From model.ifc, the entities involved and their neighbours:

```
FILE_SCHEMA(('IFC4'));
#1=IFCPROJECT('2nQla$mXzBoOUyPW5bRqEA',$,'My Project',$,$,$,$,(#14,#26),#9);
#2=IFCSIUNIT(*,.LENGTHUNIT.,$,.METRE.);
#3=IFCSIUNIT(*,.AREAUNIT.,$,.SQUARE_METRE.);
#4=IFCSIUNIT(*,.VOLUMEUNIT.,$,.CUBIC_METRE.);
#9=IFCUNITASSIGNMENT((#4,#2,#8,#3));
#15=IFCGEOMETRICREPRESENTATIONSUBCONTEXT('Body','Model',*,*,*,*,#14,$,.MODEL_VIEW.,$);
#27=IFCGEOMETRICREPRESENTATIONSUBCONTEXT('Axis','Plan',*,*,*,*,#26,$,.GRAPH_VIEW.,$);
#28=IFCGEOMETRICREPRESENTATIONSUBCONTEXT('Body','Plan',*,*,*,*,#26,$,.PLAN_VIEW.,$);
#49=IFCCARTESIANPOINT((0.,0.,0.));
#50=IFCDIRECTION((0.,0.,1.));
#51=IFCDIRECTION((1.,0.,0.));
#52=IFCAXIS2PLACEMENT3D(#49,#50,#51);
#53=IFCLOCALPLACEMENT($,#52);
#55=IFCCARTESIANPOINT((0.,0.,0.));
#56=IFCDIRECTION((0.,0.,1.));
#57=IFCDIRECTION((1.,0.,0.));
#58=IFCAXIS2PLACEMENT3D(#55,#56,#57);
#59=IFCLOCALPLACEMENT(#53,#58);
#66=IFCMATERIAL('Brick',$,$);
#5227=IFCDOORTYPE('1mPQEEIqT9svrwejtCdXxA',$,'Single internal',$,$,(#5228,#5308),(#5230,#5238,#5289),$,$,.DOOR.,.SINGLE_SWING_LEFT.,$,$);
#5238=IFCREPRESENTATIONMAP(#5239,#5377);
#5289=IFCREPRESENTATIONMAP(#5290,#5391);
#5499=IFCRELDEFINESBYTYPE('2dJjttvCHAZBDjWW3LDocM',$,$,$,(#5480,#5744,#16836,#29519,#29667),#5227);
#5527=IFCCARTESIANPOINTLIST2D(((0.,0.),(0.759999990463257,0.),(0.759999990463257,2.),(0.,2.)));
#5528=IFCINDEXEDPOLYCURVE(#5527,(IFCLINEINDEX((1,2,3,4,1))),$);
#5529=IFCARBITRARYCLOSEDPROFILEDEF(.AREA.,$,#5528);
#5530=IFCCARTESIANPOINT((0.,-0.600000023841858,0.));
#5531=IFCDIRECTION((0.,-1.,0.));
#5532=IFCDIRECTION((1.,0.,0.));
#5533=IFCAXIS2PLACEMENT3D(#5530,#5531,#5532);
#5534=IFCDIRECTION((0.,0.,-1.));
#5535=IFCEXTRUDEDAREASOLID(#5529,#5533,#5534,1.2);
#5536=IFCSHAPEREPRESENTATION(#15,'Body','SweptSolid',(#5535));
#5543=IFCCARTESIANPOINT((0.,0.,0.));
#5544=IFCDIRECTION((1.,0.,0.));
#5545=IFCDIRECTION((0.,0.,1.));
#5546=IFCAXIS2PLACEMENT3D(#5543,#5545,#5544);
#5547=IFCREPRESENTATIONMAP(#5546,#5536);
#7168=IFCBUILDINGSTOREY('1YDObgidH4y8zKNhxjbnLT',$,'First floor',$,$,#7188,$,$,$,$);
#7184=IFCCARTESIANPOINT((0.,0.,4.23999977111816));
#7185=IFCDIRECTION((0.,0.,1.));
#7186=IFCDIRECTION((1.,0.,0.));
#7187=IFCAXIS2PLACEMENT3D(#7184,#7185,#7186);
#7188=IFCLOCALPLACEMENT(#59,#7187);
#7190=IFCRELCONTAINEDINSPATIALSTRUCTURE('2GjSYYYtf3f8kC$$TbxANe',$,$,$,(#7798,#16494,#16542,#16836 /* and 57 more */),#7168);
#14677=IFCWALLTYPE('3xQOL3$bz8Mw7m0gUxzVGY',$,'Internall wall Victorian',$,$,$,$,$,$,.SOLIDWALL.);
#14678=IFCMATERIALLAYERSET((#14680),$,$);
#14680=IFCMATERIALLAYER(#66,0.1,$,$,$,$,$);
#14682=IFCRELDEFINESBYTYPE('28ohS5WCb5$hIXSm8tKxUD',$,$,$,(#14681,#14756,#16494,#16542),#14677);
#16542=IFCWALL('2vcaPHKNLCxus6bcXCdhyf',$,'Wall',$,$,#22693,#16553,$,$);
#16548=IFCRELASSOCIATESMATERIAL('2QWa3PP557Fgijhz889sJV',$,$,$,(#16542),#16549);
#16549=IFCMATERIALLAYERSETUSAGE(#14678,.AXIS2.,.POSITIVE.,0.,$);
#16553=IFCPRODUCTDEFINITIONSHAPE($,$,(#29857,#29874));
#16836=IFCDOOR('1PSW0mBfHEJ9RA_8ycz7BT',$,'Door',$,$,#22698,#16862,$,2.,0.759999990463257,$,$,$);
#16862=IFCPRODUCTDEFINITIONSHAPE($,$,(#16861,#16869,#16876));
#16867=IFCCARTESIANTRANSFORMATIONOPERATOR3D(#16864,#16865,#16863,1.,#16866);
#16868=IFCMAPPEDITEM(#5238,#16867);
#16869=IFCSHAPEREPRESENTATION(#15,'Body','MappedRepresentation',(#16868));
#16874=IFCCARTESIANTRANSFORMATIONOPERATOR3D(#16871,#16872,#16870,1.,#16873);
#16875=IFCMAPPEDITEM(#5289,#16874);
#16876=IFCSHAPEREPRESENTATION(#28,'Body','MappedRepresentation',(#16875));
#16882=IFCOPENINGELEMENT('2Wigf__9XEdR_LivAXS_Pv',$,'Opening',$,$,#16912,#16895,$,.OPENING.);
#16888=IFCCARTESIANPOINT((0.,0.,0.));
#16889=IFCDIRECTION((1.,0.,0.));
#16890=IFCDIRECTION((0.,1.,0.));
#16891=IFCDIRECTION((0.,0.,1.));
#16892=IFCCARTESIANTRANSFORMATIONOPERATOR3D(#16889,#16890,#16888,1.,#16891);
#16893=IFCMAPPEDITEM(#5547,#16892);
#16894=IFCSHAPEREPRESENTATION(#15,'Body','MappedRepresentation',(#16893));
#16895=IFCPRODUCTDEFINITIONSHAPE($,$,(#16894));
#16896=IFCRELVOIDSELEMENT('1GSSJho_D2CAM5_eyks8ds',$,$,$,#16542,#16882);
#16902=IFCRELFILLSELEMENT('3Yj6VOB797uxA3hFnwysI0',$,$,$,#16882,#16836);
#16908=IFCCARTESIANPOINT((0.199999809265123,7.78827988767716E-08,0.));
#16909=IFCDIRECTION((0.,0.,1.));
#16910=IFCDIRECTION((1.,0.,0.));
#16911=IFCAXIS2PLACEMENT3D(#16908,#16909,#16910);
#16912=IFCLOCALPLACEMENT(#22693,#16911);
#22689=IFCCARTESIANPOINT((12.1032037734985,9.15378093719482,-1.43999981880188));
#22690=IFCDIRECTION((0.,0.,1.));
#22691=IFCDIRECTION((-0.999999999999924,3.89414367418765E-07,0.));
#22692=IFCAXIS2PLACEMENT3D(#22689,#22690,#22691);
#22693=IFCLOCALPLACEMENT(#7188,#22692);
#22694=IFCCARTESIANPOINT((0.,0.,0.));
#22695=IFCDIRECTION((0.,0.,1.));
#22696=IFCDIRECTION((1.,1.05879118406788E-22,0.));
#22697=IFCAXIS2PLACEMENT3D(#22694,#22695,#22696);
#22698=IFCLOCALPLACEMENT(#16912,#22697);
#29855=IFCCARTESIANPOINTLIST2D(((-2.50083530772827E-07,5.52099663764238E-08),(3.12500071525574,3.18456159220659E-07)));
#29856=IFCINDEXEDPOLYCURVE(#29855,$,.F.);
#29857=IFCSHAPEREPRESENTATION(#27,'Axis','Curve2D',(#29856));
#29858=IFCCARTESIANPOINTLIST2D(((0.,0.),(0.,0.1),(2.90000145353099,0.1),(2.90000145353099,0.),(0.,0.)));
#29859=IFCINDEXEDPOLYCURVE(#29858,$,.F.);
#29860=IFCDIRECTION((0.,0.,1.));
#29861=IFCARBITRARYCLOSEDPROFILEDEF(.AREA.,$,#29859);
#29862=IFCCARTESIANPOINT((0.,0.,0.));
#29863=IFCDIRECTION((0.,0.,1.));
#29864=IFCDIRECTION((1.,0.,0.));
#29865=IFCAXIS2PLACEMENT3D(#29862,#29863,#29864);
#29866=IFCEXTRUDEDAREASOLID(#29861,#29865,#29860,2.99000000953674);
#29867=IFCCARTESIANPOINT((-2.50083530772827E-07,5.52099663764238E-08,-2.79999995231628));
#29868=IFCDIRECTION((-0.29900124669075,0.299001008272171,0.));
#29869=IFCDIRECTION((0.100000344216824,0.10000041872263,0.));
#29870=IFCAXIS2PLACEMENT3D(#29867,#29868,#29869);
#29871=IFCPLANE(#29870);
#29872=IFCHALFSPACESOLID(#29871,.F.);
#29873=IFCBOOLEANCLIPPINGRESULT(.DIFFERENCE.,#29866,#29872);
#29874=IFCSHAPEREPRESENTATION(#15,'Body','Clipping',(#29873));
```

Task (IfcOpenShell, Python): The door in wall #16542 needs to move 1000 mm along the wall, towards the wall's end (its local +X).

```python
import ifcopenshell
import ifcopenshell.api.geometry
import ifcopenshell.util.placement
import ifcopenshell.util.unit

model = ifcopenshell.open("model.ifc")
unit_scale = ifcopenshell.util.unit.calculate_unit_scale(model)

door = model.by_id(16836)
opening = door.FillsVoids[0].RelatingOpeningElement
wall = opening.VoidsElements[0].RelatingBuildingElement

wall_matrix = ifcopenshell.util.placement.get_local_placement(wall.ObjectPlacement)
shift = wall_matrix[:3, 0] * 1 / unit_scale
before = ifcopenshell.util.placement.get_local_placement(door.ObjectPlacement)[:3, 3].copy()

# The door is placed relative to its opening, so it follows when the opening moves.
matrix = ifcopenshell.util.placement.get_local_placement(opening.ObjectPlacement)
matrix[:3, 3] += shift
ifcopenshell.api.geometry.edit_object_placement(
    model, product=opening, matrix=matrix, is_si=False, should_transform_children=True
)

after = ifcopenshell.util.placement.get_local_placement(door.ObjectPlacement)[:3, 3]
print("door moved by", (after - before).round(3) + 0.0)

model.write("model_v2.ifc")
```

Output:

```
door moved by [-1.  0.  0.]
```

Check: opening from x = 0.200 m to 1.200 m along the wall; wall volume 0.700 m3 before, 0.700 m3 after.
